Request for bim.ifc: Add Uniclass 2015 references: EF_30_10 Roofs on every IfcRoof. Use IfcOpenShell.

First a look at what the model holds.

```python
import ifcopenshell

model = ifcopenshell.open("bim.ifc")
print(model.schema)
print("classifications:", [c.Name for c in model.by_type("IfcClassification")])
for ifc_class in ("IfcDoor", "IfcRoof", "IfcStair", "IfcWall", "IfcWindow"):
    print(ifc_class, len(model.by_type(ifc_class)))
```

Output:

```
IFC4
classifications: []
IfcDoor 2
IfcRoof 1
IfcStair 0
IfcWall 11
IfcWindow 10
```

```python
import ifcopenshell
import ifcopenshell.api.classification

model = ifcopenshell.open("bim.ifc")

system = ifcopenshell.api.classification.add_classification(model, classification="Uniclass 2015")

codes = {
    "IfcRoof": ("EF_30_10", "Roofs"),
}
for ifc_class, (code, name) in codes.items():
    products = model.by_type(ifc_class)
    ifcopenshell.api.classification.add_reference(
        model, products=products, classification=system, identification=code, name=name
    )
    print(code, len(products))

model.write("bim_updated.ifc")
```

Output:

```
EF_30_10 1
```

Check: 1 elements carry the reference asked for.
